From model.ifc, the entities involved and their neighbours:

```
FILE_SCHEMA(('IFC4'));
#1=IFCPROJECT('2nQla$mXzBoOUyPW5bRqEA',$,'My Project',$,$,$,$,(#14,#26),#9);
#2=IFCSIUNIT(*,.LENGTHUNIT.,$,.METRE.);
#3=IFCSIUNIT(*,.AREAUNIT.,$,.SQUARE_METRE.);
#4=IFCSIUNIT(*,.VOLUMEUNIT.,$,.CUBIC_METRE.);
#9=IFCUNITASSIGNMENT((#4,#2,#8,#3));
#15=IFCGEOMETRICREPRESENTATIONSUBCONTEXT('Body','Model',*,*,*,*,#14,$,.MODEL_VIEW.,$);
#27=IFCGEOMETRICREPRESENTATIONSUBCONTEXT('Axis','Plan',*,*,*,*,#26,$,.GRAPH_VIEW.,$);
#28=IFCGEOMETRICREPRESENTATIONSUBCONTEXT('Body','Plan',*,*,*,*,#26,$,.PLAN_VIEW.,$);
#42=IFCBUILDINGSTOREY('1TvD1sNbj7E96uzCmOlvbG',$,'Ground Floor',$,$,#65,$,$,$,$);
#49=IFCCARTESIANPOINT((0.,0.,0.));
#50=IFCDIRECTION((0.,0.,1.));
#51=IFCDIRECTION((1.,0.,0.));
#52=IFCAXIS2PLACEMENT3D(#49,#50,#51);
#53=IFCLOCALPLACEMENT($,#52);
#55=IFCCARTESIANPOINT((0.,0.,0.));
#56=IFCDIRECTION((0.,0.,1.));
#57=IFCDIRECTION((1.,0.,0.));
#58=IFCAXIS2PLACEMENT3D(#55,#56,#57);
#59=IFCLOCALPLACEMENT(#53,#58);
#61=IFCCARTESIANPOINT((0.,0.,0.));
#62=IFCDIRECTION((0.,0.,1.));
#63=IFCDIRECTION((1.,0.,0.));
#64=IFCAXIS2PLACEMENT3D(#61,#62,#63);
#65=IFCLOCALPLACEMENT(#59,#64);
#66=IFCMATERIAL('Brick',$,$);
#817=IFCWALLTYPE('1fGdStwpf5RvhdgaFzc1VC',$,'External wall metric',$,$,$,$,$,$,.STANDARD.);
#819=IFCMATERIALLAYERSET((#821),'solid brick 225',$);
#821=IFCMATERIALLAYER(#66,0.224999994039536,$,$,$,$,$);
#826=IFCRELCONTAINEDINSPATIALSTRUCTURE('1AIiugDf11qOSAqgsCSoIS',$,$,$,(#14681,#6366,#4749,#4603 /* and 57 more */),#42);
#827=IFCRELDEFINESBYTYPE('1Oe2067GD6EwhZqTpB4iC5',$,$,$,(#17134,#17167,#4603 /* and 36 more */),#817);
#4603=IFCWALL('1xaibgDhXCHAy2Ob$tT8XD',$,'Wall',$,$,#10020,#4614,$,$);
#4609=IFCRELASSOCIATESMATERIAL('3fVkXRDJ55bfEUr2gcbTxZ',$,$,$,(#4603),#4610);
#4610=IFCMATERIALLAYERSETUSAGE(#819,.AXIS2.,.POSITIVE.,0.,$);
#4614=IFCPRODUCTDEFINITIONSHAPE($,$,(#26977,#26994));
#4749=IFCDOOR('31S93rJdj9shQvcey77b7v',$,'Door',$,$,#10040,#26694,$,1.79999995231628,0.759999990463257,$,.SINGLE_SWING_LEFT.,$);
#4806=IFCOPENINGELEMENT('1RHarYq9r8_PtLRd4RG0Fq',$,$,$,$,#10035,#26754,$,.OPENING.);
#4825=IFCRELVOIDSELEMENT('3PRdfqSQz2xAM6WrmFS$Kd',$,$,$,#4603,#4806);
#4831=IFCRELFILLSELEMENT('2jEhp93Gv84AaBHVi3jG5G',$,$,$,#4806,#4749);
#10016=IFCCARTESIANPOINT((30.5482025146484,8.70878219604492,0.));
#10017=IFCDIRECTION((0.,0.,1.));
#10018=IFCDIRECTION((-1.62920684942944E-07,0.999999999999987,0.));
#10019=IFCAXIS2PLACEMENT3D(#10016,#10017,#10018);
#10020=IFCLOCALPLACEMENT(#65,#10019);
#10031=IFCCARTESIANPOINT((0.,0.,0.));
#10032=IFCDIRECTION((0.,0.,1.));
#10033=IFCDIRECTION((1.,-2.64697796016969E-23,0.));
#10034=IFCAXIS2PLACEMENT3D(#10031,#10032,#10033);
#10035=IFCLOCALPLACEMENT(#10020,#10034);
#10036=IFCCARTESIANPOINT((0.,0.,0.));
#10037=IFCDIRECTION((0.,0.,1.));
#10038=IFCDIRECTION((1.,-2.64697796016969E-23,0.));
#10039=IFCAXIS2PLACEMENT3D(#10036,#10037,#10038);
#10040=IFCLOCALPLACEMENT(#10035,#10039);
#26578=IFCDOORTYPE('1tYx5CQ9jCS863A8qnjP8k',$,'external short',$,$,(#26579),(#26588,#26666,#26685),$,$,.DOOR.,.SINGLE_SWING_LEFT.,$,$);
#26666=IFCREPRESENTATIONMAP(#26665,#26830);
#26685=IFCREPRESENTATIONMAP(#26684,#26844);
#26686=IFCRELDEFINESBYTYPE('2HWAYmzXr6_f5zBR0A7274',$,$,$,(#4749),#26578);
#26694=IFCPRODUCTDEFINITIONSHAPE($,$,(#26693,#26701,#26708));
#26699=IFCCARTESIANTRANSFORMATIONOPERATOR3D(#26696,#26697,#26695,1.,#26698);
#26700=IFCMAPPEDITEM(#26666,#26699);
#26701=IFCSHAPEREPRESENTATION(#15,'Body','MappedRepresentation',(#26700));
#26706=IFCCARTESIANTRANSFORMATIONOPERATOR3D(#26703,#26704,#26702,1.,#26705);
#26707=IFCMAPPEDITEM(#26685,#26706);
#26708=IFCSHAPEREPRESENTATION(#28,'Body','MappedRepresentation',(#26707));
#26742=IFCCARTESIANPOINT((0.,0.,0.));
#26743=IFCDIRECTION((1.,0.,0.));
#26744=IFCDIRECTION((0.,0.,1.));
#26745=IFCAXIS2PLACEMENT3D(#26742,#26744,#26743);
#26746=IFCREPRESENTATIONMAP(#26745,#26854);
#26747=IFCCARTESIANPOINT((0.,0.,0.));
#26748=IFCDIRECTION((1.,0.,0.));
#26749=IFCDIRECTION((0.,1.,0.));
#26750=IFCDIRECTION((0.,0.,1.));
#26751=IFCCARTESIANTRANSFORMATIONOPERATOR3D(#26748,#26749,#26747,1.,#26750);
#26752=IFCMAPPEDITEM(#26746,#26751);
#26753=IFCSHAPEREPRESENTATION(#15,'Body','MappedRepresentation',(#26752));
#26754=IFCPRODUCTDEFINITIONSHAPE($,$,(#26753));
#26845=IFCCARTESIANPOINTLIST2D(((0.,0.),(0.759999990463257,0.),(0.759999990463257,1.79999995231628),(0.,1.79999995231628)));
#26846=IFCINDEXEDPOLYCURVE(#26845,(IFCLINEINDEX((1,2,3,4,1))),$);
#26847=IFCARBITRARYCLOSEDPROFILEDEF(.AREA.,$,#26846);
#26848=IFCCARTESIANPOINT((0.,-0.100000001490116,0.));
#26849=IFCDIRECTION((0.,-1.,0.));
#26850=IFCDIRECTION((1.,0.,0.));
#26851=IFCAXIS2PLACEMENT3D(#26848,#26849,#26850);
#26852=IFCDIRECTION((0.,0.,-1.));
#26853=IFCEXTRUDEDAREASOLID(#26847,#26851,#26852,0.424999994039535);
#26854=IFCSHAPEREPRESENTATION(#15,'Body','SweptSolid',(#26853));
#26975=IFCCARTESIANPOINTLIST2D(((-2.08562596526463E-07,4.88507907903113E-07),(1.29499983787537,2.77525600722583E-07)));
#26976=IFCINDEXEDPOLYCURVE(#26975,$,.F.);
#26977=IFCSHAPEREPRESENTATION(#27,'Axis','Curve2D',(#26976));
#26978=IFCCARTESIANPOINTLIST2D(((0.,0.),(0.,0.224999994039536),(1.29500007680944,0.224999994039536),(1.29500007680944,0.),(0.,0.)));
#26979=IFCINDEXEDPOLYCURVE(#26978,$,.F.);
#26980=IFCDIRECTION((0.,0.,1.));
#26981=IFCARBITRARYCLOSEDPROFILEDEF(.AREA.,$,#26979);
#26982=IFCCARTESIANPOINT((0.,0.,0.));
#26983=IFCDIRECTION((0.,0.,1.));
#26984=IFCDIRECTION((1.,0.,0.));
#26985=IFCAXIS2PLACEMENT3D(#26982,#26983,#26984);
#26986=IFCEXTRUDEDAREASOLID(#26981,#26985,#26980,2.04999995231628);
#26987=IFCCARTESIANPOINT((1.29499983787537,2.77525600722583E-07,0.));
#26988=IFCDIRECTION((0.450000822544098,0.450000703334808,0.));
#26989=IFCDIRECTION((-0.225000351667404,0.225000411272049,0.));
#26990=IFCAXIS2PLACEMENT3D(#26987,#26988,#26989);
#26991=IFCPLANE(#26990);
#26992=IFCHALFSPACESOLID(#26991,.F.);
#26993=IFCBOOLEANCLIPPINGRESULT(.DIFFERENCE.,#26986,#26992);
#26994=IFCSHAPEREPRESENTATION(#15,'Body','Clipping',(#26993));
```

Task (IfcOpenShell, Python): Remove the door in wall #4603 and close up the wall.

```python
import ifcopenshell
import ifcopenshell.api.feature
import ifcopenshell.api.root
import ifcopenshell.geom
import ifcopenshell.util.shape

model = ifcopenshell.open("model.ifc")
settings = ifcopenshell.geom.settings()


def volume(element):
    """Net volume in cubic metres, openings subtracted."""
    shape = ifcopenshell.geom.create_shape(settings, element)
    return ifcopenshell.util.shape.get_volume(shape.geometry)


door = model.by_guid("31S93rJdj9shQvcey77b7v")
opening = door.FillsVoids[0].RelatingOpeningElement
wall = opening.VoidsElements[0].RelatingBuildingElement
before = volume(wall)

ifcopenshell.api.root.remove_product(model, product=door)
ifcopenshell.api.feature.remove_feature(model, feature=opening)

after = volume(wall)

print(f"wall volume {before:.3f} -> {after:.3f} m3")

model.write("model_edited.ifc")
```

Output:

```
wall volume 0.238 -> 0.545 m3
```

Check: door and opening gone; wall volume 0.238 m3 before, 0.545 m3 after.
